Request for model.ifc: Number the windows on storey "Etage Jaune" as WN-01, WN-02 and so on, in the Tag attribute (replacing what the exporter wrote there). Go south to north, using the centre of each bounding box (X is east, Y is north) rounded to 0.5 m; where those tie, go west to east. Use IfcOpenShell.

First a look at what the model holds.

```python
import ifcopenshell
import ifcopenshell.util.element
import ifcopenshell.util.placement

model = ifcopenshell.open("model.ifc")
print(model.schema)
storey = next(s for s in model.by_type("IfcBuildingStorey") if s.Name == "Etage Jaune")
windows = [e for e in ifcopenshell.util.element.get_decomposition(storey) if e.is_a("IfcWindow")]
for e in sorted(windows, key=lambda e: e.id()):
    origin = ifcopenshell.util.placement.get_local_placement(e.ObjectPlacement)[:3, 3]
    print(e.id(), e.Tag, e.Name, origin.round(2) + 0.0, sep=" | ")
```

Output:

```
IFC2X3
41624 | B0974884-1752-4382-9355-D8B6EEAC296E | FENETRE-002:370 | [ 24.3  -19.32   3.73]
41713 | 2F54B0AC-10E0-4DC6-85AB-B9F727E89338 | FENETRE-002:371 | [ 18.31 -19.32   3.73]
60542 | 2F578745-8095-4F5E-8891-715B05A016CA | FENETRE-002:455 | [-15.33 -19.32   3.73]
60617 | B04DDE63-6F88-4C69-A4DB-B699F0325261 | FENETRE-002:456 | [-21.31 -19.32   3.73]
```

```python
import ifcopenshell
import ifcopenshell.geom
import ifcopenshell.util.element
import ifcopenshell.util.shape

model = ifcopenshell.open("model.ifc")
settings = ifcopenshell.geom.settings()
settings.set("use-world-coords", True)


def centre(element):
    shape = ifcopenshell.geom.create_shape(settings, element)
    return ifcopenshell.util.shape.get_bbox_centroid(shape.geometry)


storey = next(s for s in model.by_type("IfcBuildingStorey") if s.Name == "Etage Jaune")
windows = [e for e in ifcopenshell.util.element.get_decomposition(storey) if e.is_a("IfcWindow")]

# Insertion points can sit at a corner or the storey origin, so sort by the geometry (in metres).
centres = {e: centre(e) for e in windows}
windows.sort(key=lambda e: (round(centres[e][1] / 0.5), centres[e][0]))

for i, e in enumerate(windows, start=1):
    number = f"WN-{i:02d}"
    e.Tag = number
    print(e.id(), number)

model.write("model_updated.ifc")
```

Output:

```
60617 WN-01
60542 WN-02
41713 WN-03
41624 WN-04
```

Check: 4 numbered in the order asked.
